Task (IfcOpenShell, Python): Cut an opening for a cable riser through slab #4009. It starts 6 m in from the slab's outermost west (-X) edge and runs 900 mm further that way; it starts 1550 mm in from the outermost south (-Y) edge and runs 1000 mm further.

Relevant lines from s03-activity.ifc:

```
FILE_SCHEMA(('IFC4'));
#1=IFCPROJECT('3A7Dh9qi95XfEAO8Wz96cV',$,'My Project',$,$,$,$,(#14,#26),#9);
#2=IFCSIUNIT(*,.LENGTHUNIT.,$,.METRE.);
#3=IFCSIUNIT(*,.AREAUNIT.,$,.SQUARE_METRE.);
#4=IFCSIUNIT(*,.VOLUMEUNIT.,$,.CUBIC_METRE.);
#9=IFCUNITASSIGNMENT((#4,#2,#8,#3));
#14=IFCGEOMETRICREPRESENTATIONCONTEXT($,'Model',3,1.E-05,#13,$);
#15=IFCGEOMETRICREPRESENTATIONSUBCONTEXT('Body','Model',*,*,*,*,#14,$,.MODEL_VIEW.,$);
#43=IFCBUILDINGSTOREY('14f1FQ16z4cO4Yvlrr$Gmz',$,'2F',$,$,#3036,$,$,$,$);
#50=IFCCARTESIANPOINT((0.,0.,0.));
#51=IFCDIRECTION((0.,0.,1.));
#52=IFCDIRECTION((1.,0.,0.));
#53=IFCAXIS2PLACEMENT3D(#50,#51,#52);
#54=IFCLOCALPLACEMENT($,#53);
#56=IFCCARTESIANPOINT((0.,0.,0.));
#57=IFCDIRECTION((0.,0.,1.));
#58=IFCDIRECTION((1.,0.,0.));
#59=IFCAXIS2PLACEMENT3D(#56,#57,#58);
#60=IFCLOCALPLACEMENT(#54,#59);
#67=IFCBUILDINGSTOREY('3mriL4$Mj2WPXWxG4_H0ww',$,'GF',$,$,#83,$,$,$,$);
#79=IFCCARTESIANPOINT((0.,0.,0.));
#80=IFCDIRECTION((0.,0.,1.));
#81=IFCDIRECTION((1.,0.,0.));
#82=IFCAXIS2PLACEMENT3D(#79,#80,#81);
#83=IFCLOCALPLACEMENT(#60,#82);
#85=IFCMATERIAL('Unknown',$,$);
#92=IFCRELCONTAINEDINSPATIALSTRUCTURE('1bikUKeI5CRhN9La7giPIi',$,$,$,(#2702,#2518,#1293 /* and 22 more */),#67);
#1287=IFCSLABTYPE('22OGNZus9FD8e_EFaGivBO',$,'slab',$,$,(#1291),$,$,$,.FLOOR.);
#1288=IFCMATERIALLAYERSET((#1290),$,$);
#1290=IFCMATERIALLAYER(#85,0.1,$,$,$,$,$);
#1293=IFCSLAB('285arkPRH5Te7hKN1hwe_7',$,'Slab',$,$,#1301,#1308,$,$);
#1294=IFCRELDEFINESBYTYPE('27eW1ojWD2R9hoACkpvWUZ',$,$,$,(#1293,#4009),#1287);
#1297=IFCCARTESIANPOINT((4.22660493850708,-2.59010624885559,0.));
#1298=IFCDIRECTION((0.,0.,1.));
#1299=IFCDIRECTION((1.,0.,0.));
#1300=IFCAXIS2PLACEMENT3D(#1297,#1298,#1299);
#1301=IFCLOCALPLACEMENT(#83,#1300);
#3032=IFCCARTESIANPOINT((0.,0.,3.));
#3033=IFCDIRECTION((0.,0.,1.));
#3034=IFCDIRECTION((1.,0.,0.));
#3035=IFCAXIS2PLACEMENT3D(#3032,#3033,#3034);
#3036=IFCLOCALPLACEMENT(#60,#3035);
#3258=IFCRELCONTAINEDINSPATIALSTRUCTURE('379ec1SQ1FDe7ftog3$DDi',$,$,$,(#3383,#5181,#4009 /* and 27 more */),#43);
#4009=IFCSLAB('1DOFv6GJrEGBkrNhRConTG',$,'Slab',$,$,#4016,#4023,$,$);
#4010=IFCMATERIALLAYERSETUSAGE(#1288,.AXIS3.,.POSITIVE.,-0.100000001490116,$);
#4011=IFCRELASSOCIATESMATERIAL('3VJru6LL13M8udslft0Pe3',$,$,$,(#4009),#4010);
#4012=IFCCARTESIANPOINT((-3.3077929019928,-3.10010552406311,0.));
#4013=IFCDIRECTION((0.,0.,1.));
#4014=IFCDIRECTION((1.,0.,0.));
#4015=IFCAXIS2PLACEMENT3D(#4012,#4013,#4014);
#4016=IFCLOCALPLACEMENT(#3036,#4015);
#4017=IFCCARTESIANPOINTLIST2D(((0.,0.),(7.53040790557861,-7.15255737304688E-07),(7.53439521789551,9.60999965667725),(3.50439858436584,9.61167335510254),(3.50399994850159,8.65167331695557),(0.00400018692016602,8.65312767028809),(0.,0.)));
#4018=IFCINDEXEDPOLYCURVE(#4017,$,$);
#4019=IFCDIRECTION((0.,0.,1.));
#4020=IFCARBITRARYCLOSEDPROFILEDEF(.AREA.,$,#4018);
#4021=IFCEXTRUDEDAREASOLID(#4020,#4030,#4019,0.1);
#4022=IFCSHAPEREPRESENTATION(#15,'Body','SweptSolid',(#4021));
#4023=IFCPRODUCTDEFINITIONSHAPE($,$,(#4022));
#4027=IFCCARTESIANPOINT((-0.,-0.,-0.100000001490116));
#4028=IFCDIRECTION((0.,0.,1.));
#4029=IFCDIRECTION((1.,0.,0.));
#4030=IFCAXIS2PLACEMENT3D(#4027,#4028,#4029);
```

```python
import numpy as np
import ifcopenshell
import ifcopenshell.api.feature
import ifcopenshell.api.geometry
import ifcopenshell.api.root
import ifcopenshell.geom
import ifcopenshell.util.placement
import ifcopenshell.util.representation
import ifcopenshell.util.shape
import ifcopenshell.util.unit

model = ifcopenshell.open("s03-activity.ifc")
unit_scale = ifcopenshell.util.unit.calculate_unit_scale(model)
settings = ifcopenshell.geom.settings()


def volume(element):
    """Net volume in cubic metres, openings subtracted."""
    shape = ifcopenshell.geom.create_shape(settings, element)
    return ifcopenshell.util.shape.get_volume(shape.geometry)


slab = model.by_guid("1DOFv6GJrEGBkrNhRConTG")
before = volume(slab)

# Extent in the slab's own axes, in metres. The edges named are its -X and -Y sides.
slab_shape = ifcopenshell.geom.create_shape(settings, slab)
vertices = ifcopenshell.util.shape.get_vertices(slab_shape.geometry)
x_min, y_min, bottom = vertices.min(axis=0)
top = vertices[:, 2].max()

opening = ifcopenshell.api.root.create_entity(model, ifc_class="IfcOpeningElement", name="Cable riser opening", predefined_type="OPENING")
context = ifcopenshell.util.representation.get_context(model, "Model", "Body", "MODEL_VIEW")
width, depth = 0.9, 1
outline = [(0.0, 0.0), (width, 0.0), (width, depth), (0.0, depth), (0.0, 0.0)]
# Overshoot both faces by 50 mm so the cut is clean.
shape = ifcopenshell.api.geometry.add_slab_representation(
    model, context=context, depth=top - bottom + 0.1, polyline=outline
)
ifcopenshell.api.geometry.assign_representation(model, product=opening, representation=shape)

matrix = ifcopenshell.util.placement.get_local_placement(slab.ObjectPlacement)
matrix[:, 3] = matrix @ np.append(np.array([x_min + 6, y_min + 1.55, bottom - 0.05]) / unit_scale, 1.0)
ifcopenshell.api.geometry.edit_object_placement(model, product=opening, matrix=matrix, is_si=False)
ifcopenshell.api.feature.add_feature(model, feature=opening, element=slab)

after = volume(slab)

print(f"slab volume {before:.3f} -> {after:.3f} m3")

model.write("s03-activity_edited.ifc")
```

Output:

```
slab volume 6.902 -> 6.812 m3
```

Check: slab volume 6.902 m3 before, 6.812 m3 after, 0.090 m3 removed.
